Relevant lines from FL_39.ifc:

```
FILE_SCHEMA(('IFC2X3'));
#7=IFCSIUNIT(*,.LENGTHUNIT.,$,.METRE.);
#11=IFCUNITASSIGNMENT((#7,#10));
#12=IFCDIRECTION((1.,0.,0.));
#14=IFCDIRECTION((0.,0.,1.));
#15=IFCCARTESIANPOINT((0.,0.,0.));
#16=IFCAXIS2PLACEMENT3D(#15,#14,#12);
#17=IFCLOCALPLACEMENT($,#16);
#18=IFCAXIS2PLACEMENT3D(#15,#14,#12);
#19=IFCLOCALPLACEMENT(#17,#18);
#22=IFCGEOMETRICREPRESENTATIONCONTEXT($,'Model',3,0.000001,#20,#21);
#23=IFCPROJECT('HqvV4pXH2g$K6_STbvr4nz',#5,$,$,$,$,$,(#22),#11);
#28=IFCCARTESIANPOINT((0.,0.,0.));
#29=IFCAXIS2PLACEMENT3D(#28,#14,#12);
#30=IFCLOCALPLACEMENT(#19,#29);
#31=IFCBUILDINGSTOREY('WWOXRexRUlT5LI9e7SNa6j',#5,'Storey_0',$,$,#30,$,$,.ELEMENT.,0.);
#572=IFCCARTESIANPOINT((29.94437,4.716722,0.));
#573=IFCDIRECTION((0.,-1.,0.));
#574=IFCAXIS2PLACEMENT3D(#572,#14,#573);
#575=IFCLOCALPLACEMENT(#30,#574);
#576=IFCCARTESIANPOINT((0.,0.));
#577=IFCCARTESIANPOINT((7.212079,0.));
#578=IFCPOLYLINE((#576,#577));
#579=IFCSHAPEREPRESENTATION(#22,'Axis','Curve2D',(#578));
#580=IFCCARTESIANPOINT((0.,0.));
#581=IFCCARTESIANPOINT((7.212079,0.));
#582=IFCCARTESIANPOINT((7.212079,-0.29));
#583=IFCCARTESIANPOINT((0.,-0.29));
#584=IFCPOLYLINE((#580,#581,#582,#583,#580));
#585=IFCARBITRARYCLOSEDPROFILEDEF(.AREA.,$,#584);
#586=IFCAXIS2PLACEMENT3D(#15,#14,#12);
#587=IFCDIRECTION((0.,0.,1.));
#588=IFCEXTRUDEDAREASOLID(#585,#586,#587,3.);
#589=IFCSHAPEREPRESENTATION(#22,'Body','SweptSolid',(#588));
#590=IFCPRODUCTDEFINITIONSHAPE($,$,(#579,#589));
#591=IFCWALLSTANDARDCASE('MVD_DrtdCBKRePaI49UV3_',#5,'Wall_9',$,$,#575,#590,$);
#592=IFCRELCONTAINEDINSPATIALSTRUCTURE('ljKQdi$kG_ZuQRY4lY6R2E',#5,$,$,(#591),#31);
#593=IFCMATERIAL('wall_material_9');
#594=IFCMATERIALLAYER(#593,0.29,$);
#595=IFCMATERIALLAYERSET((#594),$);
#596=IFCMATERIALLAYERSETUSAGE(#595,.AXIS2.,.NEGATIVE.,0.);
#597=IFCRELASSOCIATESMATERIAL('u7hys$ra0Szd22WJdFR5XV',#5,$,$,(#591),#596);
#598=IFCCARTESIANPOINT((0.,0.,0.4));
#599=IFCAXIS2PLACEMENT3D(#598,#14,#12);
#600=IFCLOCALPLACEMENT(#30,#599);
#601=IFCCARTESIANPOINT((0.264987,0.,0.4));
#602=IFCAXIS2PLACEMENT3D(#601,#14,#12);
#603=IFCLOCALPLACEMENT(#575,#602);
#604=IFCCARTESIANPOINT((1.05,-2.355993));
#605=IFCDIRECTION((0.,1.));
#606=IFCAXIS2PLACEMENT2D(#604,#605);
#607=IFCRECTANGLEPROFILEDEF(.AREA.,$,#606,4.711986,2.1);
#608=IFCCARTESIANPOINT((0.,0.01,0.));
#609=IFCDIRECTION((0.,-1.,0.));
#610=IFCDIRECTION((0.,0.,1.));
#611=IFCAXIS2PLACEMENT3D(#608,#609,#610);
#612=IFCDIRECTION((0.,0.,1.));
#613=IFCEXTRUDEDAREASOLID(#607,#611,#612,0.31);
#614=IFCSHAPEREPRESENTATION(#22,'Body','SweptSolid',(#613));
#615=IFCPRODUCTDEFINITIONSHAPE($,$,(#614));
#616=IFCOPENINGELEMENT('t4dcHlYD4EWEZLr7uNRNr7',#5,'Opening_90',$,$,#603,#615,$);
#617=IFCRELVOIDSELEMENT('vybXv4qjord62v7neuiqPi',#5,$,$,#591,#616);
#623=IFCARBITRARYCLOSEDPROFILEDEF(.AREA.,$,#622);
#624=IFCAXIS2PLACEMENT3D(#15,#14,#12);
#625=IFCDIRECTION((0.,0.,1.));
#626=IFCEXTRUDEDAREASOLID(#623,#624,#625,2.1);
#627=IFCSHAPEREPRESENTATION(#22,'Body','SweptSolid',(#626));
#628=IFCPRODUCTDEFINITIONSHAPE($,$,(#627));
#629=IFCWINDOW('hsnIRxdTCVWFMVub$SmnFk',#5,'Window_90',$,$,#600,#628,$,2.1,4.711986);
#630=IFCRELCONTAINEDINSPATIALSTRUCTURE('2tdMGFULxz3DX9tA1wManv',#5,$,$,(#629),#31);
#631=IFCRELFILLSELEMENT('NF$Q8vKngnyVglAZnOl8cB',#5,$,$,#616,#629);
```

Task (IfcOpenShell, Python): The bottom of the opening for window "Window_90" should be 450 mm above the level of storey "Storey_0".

```python
import numpy as np
import ifcopenshell
import ifcopenshell.api.geometry
import ifcopenshell.geom
import ifcopenshell.util.element
import ifcopenshell.util.placement
import ifcopenshell.util.shape
import ifcopenshell.util.unit

model = ifcopenshell.open("FL_39.ifc")
unit_scale = ifcopenshell.util.unit.calculate_unit_scale(model)

window = model.by_guid("hsnIRxdTCVWFMVub$SmnFk")
opening = window.FillsVoids[0].RelatingOpeningElement
storey = ifcopenshell.util.element.get_container(window, ifc_class="IfcBuildingStorey")
level = ifcopenshell.util.placement.get_local_placement(storey.ObjectPlacement)[2, 3]

# The opening's origin need not be at the sill, so measure its lowest point.
shape = ifcopenshell.geom.create_shape(ifcopenshell.geom.settings(), opening)
bottom = ifcopenshell.util.shape.get_shape_bottom_elevation(shape, shape.geometry) / unit_scale
dz = level + 0.45 / unit_scale - bottom

shift = np.array([0.0, 0.0, dz])
# The window is not placed relative to its opening, so move both.
for product in (opening, window):
    matrix = ifcopenshell.util.placement.get_local_placement(product.ObjectPlacement)
    matrix[:3, 3] += shift
    ifcopenshell.api.geometry.edit_object_placement(model, product=product, matrix=matrix, is_si=False)

print(f"moved by {dz * unit_scale:+.3f} m")

model.write("FL_39-out.ifc")
```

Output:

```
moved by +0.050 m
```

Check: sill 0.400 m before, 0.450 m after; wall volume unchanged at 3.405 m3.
